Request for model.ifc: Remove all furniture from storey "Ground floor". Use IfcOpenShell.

First a look at what the model holds.

```python
import ifcopenshell
import ifcopenshell.util.element

model = ifcopenshell.open("model.ifc")
print(model.schema)
storey = next(s for s in model.by_type("IfcBuildingStorey") if s.Name == "Ground floor")
furniture = [e for e in ifcopenshell.util.element.get_decomposition(storey) if e.is_a("IfcFurnishingElement")]
seen = {}
for e in furniture:
    element_type = ifcopenshell.util.element.get_type(e)
    name = element_type.Name if element_type not in (None, e) else None
    seen[name] = seen.get(name, 0) + 1
for name, count in sorted(seen.items(), key=str):
    print(count, "x", name)
```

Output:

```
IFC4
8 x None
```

```python
import ifcopenshell
import ifcopenshell.api.root
import ifcopenshell.util.element

model = ifcopenshell.open("model.ifc")

storey = next(s for s in model.by_type("IfcBuildingStorey") if s.Name == "Ground floor")
furniture = [e for e in ifcopenshell.util.element.get_decomposition(storey) if e.is_a("IfcFurnishingElement")]

for e in furniture:
    ifcopenshell.api.root.remove_product(model, product=e)
print(len(furniture), "removed")

model.write("model-out.ifc")
```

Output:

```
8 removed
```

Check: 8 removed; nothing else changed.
